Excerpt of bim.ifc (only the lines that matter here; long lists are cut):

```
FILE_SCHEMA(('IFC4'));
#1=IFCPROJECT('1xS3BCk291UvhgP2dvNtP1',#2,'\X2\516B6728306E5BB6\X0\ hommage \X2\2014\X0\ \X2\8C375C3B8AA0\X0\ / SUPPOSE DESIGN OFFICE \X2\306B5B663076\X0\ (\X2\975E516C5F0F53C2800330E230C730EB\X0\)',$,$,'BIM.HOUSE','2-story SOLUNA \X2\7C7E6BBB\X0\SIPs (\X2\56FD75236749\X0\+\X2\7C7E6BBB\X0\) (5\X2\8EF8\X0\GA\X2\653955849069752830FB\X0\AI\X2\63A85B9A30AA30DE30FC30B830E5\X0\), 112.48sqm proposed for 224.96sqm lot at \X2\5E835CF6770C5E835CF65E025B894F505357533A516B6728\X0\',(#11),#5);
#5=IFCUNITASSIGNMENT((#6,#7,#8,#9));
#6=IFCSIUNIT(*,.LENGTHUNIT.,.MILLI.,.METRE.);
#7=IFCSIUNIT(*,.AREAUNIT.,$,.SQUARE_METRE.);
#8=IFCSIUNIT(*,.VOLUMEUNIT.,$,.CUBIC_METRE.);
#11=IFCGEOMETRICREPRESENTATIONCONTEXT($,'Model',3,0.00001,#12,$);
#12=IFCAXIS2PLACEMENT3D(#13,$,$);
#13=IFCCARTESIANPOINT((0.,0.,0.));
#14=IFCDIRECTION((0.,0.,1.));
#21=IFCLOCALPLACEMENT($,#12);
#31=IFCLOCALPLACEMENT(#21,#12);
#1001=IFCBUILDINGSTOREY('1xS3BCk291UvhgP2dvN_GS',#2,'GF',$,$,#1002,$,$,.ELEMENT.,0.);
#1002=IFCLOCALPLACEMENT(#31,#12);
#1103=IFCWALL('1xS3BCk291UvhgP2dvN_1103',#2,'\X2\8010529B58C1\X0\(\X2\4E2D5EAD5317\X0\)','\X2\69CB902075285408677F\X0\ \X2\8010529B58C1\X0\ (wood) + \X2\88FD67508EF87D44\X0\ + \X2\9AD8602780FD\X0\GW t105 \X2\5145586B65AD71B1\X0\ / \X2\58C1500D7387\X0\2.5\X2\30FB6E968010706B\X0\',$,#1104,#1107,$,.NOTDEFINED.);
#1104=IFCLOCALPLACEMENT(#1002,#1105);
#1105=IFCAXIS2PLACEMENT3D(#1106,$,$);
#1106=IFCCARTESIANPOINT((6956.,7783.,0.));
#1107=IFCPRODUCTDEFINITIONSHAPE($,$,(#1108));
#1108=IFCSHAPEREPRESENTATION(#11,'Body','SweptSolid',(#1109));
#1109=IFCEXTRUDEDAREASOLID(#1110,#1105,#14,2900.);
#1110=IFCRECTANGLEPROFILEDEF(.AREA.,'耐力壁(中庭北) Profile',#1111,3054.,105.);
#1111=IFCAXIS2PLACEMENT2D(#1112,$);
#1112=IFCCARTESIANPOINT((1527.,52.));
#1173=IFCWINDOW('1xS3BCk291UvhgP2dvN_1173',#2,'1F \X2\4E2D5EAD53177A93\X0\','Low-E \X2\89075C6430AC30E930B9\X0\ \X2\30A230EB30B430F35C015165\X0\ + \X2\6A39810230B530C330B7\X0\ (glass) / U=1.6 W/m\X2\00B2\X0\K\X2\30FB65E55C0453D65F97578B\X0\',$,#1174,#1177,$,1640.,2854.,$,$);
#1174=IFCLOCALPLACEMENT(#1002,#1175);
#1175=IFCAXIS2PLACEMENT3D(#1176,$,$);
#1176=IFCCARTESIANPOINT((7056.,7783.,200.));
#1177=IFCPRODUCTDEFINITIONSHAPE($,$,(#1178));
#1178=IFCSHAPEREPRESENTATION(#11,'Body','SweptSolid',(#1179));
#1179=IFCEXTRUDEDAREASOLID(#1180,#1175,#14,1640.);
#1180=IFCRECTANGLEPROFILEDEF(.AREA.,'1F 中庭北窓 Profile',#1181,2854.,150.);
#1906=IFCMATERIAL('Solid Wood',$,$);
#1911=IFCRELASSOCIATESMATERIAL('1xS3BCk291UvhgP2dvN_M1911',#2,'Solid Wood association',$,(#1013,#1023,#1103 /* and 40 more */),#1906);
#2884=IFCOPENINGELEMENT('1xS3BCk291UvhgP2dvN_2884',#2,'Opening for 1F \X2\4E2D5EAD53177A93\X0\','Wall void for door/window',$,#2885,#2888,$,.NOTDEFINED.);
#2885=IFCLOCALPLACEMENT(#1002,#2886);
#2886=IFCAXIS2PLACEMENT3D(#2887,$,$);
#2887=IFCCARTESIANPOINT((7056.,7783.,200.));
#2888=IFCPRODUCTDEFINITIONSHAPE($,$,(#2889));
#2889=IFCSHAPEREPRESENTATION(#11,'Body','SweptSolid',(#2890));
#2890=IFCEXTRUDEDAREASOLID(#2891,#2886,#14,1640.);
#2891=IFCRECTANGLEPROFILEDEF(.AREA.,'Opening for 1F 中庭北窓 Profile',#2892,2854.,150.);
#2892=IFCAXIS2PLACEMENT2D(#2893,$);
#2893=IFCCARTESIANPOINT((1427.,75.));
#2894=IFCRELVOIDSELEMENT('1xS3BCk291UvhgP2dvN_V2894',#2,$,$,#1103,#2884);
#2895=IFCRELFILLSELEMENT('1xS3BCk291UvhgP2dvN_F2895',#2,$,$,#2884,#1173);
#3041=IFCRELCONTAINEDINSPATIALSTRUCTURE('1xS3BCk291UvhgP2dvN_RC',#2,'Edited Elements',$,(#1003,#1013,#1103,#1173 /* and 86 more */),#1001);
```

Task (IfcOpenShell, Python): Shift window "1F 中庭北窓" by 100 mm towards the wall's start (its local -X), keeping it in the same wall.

```python
import ifcopenshell
import ifcopenshell.api.geometry
import ifcopenshell.util.placement
import ifcopenshell.util.unit

model = ifcopenshell.open("bim.ifc")
unit_scale = ifcopenshell.util.unit.calculate_unit_scale(model)

window = model.by_id(1173)
opening = window.FillsVoids[0].RelatingOpeningElement
wall = opening.VoidsElements[0].RelatingBuildingElement

wall_matrix = ifcopenshell.util.placement.get_local_placement(wall.ObjectPlacement)
shift = wall_matrix[:3, 0] * -0.1 / unit_scale
before = ifcopenshell.util.placement.get_local_placement(window.ObjectPlacement)[:3, 3].copy()

# The window is not placed relative to its opening, so move both.
for product in (opening, window):
    matrix = ifcopenshell.util.placement.get_local_placement(product.ObjectPlacement)
    matrix[:3, 3] += shift
    ifcopenshell.api.geometry.edit_object_placement(model, product=product, matrix=matrix, is_si=False)

after = ifcopenshell.util.placement.get_local_placement(window.ObjectPlacement)[:3, 3]
print("window moved by", (after - before).round(3) + 0.0)

model.write("bim_updated.ifc")
```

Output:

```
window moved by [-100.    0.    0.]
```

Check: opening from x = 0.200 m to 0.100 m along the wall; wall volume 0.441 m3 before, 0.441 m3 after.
